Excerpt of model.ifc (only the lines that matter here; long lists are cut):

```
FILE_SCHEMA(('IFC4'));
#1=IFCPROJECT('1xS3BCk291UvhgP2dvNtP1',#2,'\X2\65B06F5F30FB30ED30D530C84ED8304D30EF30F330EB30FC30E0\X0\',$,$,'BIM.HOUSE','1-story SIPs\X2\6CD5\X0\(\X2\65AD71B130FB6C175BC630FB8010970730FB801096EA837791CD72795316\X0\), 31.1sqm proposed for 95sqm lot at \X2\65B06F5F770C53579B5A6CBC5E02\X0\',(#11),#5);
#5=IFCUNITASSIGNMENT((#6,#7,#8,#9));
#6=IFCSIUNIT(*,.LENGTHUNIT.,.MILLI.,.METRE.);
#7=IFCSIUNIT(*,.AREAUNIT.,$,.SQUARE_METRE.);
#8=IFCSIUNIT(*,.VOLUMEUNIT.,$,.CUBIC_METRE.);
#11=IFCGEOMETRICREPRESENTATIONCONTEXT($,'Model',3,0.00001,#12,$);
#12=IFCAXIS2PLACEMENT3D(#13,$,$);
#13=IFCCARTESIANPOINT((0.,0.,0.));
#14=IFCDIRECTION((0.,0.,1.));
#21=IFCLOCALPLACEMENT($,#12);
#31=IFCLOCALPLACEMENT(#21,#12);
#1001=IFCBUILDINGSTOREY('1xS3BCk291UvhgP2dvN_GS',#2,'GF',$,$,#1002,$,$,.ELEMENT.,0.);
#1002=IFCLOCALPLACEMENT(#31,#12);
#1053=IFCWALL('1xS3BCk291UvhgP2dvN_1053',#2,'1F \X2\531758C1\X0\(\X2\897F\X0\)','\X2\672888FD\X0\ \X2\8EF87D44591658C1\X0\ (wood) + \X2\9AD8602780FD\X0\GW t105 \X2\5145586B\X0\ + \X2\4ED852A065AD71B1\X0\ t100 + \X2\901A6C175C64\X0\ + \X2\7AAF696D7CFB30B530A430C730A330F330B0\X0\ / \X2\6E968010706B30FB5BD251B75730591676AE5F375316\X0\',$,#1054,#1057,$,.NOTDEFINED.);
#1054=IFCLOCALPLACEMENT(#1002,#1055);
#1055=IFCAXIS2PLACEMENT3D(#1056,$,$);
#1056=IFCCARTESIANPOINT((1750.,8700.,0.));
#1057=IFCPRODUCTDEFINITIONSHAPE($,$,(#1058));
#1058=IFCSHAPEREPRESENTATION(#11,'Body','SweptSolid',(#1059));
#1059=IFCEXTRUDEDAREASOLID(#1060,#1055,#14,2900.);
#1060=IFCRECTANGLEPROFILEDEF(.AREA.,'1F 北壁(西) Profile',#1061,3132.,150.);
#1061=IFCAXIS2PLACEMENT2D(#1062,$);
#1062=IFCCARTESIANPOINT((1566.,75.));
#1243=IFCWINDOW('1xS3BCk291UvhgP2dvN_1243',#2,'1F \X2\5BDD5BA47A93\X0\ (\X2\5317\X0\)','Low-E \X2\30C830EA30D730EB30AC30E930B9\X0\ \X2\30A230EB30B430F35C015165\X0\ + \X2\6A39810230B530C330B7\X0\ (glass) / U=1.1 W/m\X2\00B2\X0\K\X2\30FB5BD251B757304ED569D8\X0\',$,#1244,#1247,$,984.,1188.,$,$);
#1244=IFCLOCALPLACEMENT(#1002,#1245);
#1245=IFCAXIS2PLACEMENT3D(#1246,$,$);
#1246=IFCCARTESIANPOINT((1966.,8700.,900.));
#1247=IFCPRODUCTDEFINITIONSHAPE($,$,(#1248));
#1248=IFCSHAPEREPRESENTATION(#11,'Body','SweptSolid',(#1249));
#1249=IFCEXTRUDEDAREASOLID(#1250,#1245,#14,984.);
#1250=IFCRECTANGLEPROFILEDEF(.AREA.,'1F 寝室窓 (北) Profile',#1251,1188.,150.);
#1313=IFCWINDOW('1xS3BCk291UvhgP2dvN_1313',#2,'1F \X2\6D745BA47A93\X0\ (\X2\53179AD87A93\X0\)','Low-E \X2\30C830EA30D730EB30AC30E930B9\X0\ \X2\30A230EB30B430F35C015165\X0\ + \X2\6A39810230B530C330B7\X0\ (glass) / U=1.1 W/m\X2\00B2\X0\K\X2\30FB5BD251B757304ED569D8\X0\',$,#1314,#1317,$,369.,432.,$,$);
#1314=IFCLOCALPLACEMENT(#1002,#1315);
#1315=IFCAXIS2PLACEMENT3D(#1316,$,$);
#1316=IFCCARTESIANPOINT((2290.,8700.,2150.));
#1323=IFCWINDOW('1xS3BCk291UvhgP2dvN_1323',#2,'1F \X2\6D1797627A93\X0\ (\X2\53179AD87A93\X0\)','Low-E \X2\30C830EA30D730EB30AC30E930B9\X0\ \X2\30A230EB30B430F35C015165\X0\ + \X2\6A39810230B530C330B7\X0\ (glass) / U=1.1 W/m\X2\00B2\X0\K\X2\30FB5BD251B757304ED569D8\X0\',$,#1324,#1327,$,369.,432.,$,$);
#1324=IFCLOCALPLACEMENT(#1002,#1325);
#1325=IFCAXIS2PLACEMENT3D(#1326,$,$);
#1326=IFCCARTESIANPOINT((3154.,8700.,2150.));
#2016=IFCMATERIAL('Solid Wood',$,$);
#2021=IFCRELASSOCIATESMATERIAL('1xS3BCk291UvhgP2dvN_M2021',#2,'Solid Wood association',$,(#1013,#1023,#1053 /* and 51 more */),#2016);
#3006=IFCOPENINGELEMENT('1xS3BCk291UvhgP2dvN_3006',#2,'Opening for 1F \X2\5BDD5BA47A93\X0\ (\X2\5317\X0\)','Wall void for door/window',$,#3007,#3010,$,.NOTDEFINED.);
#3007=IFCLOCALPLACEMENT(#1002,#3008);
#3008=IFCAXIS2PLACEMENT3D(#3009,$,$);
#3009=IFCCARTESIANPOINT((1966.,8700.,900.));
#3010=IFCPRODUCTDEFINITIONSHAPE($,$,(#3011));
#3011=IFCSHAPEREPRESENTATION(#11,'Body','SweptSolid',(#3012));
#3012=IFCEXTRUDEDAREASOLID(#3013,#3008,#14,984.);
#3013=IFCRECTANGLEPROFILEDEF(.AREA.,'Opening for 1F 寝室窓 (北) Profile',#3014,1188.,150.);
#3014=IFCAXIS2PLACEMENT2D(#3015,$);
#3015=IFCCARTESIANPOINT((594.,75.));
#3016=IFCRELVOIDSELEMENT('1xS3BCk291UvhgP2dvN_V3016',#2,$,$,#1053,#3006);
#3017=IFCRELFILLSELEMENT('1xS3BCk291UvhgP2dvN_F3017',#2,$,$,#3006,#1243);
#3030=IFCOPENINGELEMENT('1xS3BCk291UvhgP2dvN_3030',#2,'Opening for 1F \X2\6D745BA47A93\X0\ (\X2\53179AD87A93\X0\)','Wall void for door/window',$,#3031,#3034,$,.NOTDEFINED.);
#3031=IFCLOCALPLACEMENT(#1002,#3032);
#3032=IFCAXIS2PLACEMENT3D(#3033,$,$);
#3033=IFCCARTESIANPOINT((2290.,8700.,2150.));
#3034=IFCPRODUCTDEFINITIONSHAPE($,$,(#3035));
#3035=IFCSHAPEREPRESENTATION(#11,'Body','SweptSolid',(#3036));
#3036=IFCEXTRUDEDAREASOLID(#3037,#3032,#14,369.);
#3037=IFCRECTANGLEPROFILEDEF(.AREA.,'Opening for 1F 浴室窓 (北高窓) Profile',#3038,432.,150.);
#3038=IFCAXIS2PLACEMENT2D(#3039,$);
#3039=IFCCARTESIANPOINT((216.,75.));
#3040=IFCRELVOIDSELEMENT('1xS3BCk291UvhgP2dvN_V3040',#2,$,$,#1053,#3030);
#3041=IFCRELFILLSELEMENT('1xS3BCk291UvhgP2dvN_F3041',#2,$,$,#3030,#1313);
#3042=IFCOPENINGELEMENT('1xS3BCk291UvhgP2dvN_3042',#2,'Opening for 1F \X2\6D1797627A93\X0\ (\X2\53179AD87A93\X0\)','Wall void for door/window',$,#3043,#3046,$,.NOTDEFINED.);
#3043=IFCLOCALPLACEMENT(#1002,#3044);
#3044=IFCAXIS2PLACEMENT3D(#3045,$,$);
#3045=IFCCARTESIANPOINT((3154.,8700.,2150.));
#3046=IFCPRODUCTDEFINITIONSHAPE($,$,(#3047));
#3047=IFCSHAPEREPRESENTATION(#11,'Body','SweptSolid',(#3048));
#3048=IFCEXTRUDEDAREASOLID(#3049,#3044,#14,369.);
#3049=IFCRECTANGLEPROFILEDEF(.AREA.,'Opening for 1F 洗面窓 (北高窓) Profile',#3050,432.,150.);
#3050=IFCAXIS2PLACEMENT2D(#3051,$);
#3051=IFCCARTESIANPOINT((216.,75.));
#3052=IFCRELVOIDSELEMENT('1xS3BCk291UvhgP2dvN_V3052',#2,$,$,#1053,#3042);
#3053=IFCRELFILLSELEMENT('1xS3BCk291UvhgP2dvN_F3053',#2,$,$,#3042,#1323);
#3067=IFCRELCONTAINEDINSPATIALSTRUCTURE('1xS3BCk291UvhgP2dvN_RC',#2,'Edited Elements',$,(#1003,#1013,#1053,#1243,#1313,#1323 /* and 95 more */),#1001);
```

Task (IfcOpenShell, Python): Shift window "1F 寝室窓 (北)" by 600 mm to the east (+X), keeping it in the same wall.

```python
import ifcopenshell
import ifcopenshell.api.geometry
import ifcopenshell.util.placement
import ifcopenshell.util.unit

model = ifcopenshell.open("model.ifc")
unit_scale = ifcopenshell.util.unit.calculate_unit_scale(model)

window = model.by_id(1243)
opening = window.FillsVoids[0].RelatingOpeningElement
wall = opening.VoidsElements[0].RelatingBuildingElement

wall_matrix = ifcopenshell.util.placement.get_local_placement(wall.ObjectPlacement)
shift = wall_matrix[:3, 0] * 0.6 / unit_scale
before = ifcopenshell.util.placement.get_local_placement(window.ObjectPlacement)[:3, 3].copy()

# The window is not placed relative to its opening, so move both.
for product in (opening, window):
    matrix = ifcopenshell.util.placement.get_local_placement(product.ObjectPlacement)
    matrix[:3, 3] += shift
    ifcopenshell.api.geometry.edit_object_placement(model, product=product, matrix=matrix, is_si=False)

after = ifcopenshell.util.placement.get_local_placement(window.ObjectPlacement)[:3, 3]
print("window moved by", (after - before).round(3) + 0.0)

model.write("model-out.ifc")
```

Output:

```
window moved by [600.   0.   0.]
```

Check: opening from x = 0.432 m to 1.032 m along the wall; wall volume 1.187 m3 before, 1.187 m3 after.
